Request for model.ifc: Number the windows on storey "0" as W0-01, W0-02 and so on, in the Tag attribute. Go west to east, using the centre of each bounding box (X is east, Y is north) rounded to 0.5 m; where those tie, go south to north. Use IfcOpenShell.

First a look at what the model holds.

```python
import ifcopenshell
import ifcopenshell.util.element
import ifcopenshell.util.placement

model = ifcopenshell.open("model.ifc")
print(model.schema)
storey = next(s for s in model.by_type("IfcBuildingStorey") if s.Name == "0")
windows = [e for e in ifcopenshell.util.element.get_decomposition(storey) if e.is_a("IfcWindow")]
for e in sorted(windows, key=lambda e: e.id()):
    origin = ifcopenshell.util.placement.get_local_placement(e.ObjectPlacement)[:3, 3]
    print(e.id(), e.Tag, e.Name, origin.round(2) + 0.0, sep=" | ")
```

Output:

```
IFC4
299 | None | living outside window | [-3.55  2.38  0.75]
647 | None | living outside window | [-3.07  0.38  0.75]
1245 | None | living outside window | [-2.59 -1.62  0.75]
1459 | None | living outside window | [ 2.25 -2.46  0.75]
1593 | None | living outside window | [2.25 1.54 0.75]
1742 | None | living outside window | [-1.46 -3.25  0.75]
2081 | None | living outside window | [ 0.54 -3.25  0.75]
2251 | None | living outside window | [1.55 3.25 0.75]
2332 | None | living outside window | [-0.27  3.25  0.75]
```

```python
import ifcopenshell
import ifcopenshell.geom
import ifcopenshell.util.element
import ifcopenshell.util.shape

model = ifcopenshell.open("model.ifc")
settings = ifcopenshell.geom.settings()
settings.set("use-world-coords", True)


def centre(element):
    shape = ifcopenshell.geom.create_shape(settings, element)
    return ifcopenshell.util.shape.get_bbox_centroid(shape.geometry)


storey = next(s for s in model.by_type("IfcBuildingStorey") if s.Name == "0")
windows = [e for e in ifcopenshell.util.element.get_decomposition(storey) if e.is_a("IfcWindow")]

# Insertion points can sit at a corner or the storey origin, so sort by the geometry (in metres).
centres = {e: centre(e) for e in windows}
windows.sort(key=lambda e: (round(centres[e][0] / 0.5), centres[e][1]))

for i, e in enumerate(windows, start=1):
    number = f"W0-{i:02d}"
    e.Tag = number
    print(e.id(), number)

model.write("model_updated.ifc")
```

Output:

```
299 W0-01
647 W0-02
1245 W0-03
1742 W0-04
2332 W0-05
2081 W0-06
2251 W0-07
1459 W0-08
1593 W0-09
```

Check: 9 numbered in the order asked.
